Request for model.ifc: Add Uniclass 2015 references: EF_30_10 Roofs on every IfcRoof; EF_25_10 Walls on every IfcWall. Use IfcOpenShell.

First a look at what the model holds.

```python
import ifcopenshell

model = ifcopenshell.open("model.ifc")
print(model.schema)
print("classifications:", [c.Name for c in model.by_type("IfcClassification")])
for ifc_class in ("IfcDoor", "IfcRoof", "IfcStair", "IfcWall", "IfcWindow"):
    print(ifc_class, len(model.by_type(ifc_class)))
```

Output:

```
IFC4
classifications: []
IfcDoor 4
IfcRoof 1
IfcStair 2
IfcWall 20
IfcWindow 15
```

```python
import ifcopenshell
import ifcopenshell.api.classification

model = ifcopenshell.open("model.ifc")

system = ifcopenshell.api.classification.add_classification(model, classification="Uniclass 2015")

codes = {
    "IfcRoof": ("EF_30_10", "Roofs"),
    "IfcWall": ("EF_25_10", "Walls"),
}
for ifc_class, (code, name) in codes.items():
    products = model.by_type(ifc_class)
    ifcopenshell.api.classification.add_reference(
        model, products=products, classification=system, identification=code, name=name
    )
    print(code, len(products))

model.write("model-out.ifc")
```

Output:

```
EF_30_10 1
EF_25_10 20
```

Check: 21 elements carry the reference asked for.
